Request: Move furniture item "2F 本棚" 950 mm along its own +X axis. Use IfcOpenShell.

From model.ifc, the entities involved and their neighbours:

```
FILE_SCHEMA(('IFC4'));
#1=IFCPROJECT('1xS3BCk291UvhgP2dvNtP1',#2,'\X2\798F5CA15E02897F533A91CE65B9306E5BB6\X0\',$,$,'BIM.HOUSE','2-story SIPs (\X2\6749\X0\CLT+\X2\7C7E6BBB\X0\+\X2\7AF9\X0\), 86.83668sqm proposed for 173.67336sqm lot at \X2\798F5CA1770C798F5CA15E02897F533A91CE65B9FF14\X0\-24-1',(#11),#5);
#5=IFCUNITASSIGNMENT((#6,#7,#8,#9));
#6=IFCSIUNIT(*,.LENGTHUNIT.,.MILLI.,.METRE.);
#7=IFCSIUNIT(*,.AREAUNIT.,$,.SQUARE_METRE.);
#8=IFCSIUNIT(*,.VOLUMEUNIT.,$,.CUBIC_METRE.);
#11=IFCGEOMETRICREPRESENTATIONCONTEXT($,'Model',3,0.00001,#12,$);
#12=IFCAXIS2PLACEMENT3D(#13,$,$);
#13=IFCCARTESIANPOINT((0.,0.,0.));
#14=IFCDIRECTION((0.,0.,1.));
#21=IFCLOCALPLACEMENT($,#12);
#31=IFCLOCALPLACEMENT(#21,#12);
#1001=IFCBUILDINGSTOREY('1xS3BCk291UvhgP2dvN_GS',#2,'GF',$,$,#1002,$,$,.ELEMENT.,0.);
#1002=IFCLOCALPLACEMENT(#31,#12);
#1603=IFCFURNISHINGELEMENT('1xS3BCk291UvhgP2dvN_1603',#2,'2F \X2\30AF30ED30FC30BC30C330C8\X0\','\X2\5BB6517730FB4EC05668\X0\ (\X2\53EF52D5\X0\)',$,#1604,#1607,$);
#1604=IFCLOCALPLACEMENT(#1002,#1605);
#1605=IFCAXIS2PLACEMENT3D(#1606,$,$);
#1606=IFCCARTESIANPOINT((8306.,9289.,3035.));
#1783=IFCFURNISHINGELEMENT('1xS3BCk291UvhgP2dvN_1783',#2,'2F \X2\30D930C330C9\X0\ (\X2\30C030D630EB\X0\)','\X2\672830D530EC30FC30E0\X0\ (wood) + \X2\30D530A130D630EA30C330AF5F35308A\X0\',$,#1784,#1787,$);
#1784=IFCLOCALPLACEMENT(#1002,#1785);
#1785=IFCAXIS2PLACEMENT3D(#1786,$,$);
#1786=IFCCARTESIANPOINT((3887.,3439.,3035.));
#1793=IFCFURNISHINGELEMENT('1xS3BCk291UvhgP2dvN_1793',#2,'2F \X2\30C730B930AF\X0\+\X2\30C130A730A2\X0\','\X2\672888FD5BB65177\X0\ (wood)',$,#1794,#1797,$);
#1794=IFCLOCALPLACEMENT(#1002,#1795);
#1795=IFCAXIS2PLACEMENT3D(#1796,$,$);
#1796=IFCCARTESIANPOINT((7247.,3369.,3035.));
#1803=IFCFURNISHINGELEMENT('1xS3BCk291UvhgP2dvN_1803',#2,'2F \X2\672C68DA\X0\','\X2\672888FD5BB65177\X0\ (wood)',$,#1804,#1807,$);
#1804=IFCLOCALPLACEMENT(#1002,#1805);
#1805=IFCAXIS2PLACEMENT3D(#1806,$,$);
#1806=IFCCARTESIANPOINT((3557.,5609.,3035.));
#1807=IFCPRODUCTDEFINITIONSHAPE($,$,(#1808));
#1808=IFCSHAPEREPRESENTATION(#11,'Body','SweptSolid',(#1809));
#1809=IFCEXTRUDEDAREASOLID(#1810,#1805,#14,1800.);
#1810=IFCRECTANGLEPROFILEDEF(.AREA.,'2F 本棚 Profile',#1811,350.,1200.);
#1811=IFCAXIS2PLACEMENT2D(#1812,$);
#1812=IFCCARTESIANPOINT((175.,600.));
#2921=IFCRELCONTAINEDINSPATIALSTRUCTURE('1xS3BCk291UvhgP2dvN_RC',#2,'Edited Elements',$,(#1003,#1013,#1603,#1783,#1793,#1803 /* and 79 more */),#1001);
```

```python
import ifcopenshell
import ifcopenshell.api.geometry
import ifcopenshell.util.placement
import ifcopenshell.util.unit

model = ifcopenshell.open("model.ifc")
unit_scale = ifcopenshell.util.unit.calculate_unit_scale(model)

item = model.by_guid("1xS3BCk291UvhgP2dvN_1803")
matrix = ifcopenshell.util.placement.get_local_placement(item.ObjectPlacement)
matrix[:3, 3] += matrix[:3, 0] * 0.95 / unit_scale
ifcopenshell.api.geometry.edit_object_placement(model, product=item, matrix=matrix, is_si=False)

print(ifcopenshell.util.placement.get_local_placement(item.ObjectPlacement).round(3) + 0.0)

model.write("model-out.ifc")
```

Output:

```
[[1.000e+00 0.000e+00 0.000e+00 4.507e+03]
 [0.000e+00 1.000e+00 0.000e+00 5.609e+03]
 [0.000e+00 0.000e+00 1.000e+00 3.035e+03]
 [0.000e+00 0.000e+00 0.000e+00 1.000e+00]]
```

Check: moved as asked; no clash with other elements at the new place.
